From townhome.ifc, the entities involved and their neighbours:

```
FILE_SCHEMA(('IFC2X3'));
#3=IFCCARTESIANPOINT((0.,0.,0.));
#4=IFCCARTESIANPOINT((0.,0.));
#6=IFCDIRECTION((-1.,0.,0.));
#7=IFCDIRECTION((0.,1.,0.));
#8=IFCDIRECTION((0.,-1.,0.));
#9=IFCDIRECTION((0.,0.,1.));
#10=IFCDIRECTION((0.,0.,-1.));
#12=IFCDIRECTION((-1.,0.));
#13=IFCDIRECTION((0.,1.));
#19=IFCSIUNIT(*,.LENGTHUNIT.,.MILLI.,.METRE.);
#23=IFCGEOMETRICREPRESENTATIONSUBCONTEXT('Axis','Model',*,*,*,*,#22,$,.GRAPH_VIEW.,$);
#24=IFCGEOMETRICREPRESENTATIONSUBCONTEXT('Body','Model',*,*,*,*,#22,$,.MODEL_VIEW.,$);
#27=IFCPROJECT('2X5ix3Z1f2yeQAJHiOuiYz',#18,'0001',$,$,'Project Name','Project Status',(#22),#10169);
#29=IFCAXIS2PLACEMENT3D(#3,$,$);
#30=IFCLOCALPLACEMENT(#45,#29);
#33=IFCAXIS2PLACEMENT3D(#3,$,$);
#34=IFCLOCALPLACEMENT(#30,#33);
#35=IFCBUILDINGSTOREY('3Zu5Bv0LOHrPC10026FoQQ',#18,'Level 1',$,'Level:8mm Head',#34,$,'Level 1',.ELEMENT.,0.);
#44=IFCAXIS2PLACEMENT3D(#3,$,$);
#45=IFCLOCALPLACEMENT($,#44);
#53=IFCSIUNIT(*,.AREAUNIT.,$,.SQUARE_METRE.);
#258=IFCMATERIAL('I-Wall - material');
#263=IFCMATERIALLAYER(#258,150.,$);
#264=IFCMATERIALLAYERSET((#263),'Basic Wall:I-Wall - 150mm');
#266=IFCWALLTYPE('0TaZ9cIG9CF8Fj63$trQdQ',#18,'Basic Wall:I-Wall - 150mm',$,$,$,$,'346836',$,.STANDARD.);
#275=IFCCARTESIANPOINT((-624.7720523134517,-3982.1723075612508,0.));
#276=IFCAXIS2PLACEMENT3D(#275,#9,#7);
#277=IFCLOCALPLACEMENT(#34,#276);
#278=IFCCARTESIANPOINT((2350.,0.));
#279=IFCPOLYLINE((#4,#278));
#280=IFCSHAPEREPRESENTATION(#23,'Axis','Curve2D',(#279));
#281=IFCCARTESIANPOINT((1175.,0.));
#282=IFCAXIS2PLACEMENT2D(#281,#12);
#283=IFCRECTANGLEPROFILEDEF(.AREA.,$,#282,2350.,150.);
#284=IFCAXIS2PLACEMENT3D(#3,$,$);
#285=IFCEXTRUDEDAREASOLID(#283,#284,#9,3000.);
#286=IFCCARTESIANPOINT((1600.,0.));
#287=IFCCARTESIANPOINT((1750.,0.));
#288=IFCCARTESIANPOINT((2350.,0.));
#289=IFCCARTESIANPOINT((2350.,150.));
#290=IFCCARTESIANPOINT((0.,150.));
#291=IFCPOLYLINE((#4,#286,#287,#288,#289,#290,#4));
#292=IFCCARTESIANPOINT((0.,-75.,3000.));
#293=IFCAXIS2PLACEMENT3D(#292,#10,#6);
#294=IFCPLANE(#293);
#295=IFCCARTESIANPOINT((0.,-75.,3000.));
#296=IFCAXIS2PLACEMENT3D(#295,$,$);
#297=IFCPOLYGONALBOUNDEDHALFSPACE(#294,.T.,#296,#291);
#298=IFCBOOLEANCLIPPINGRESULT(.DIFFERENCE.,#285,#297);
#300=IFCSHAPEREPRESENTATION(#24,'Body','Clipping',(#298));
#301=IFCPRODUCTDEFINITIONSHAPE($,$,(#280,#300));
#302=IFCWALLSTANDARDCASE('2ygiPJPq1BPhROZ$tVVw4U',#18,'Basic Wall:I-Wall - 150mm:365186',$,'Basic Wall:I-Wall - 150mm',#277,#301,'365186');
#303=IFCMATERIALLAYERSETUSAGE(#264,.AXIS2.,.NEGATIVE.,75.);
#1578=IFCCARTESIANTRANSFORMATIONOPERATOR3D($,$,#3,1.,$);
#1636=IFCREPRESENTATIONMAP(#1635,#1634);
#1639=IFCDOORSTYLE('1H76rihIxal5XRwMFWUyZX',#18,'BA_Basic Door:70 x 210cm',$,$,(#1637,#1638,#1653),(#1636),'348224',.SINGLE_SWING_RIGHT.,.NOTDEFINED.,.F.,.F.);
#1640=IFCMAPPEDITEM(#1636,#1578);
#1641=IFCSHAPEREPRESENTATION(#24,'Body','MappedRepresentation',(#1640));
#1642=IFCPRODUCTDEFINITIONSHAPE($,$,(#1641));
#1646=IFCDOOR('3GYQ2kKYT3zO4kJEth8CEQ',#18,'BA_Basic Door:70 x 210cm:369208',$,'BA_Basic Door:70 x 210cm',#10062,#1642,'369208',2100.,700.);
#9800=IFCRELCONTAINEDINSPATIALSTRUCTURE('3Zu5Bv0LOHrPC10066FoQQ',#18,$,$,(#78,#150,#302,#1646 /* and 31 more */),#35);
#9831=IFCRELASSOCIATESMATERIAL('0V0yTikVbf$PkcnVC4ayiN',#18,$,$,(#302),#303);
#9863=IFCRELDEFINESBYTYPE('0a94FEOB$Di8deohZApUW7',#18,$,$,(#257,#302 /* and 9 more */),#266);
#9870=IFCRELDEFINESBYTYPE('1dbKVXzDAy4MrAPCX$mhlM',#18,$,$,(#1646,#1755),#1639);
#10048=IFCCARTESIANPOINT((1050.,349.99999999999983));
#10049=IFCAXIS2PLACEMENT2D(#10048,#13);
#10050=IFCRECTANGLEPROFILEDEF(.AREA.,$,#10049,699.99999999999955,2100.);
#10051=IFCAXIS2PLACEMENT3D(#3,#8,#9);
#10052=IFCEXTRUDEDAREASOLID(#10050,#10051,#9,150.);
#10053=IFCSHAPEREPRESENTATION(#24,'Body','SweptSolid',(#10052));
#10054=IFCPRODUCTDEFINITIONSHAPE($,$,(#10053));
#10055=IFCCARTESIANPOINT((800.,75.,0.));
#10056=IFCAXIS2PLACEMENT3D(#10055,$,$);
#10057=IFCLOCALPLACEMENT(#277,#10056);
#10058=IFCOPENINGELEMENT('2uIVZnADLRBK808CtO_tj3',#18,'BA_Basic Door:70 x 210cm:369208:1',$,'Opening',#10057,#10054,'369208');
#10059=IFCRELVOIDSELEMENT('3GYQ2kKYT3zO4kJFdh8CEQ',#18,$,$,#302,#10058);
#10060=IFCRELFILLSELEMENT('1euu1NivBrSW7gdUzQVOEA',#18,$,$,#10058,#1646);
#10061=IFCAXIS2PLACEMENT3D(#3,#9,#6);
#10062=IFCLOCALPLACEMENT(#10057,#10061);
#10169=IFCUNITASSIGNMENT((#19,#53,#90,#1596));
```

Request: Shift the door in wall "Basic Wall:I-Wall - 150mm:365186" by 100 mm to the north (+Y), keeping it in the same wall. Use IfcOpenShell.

```python
import ifcopenshell
import ifcopenshell.api.geometry
import ifcopenshell.util.placement
import ifcopenshell.util.unit

model = ifcopenshell.open("townhome.ifc")
unit_scale = ifcopenshell.util.unit.calculate_unit_scale(model)

door = model.by_id(1646)
opening = door.FillsVoids[0].RelatingOpeningElement
wall = opening.VoidsElements[0].RelatingBuildingElement

wall_matrix = ifcopenshell.util.placement.get_local_placement(wall.ObjectPlacement)
shift = wall_matrix[:3, 0] * 0.1 / unit_scale
before = ifcopenshell.util.placement.get_local_placement(door.ObjectPlacement)[:3, 3].copy()

# The door is placed relative to its opening, so it follows when the opening moves.
matrix = ifcopenshell.util.placement.get_local_placement(opening.ObjectPlacement)
matrix[:3, 3] += shift
ifcopenshell.api.geometry.edit_object_placement(
    model, product=opening, matrix=matrix, is_si=False, should_transform_children=True
)

after = ifcopenshell.util.placement.get_local_placement(door.ObjectPlacement)[:3, 3]
print("door moved by", (after - before).round(3) + 0.0)

model.write("townhome-out.ifc")
```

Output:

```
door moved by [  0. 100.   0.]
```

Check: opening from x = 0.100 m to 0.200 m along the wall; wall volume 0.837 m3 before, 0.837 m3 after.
